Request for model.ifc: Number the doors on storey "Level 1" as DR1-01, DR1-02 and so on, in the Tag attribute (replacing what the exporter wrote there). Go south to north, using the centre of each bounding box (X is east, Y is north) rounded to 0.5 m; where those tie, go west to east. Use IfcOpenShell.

First a look at what the model holds.

```python
import ifcopenshell
import ifcopenshell.util.element
import ifcopenshell.util.placement

model = ifcopenshell.open("model.ifc")
print(model.schema)
storey = next(s for s in model.by_type("IfcBuildingStorey") if s.Name == "Level 1")
doors = [e for e in ifcopenshell.util.element.get_decomposition(storey) if e.is_a("IfcDoor")]
for e in sorted(doors, key=lambda e: e.id()):
    origin = ifcopenshell.util.placement.get_local_placement(e.ObjectPlacement)[:3, 3]
    print(e.id(), e.Tag, e.Name, origin.round(2) + 0.0, sep=" | ")
```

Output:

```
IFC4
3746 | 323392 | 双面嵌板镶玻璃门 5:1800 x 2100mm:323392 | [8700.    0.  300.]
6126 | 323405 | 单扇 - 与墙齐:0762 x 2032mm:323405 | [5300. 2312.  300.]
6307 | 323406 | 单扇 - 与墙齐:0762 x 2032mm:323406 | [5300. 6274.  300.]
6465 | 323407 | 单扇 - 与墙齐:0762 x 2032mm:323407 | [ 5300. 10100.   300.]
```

```python
import ifcopenshell
import ifcopenshell.geom
import ifcopenshell.util.element
import ifcopenshell.util.shape

model = ifcopenshell.open("model.ifc")
settings = ifcopenshell.geom.settings()
settings.set("use-world-coords", True)


def centre(element):
    shape = ifcopenshell.geom.create_shape(settings, element)
    return ifcopenshell.util.shape.get_bbox_centroid(shape.geometry)


storey = next(s for s in model.by_type("IfcBuildingStorey") if s.Name == "Level 1")
doors = [e for e in ifcopenshell.util.element.get_decomposition(storey) if e.is_a("IfcDoor")]

# Insertion points can sit at a corner or the storey origin, so sort by the geometry (in metres).
centres = {e: centre(e) for e in doors}
doors.sort(key=lambda e: (round(centres[e][1] / 0.5), centres[e][0]))

for i, e in enumerate(doors, start=1):
    number = f"DR1-{i:02d}"
    e.Tag = number
    print(e.id(), number)

model.write("model_rev.ifc")
```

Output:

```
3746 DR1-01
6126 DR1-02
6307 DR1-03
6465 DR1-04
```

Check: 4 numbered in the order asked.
